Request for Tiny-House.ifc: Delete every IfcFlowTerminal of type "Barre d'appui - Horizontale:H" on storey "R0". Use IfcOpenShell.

First a look at what the model holds.

```python
import ifcopenshell
import ifcopenshell.util.element

model = ifcopenshell.open("Tiny-House.ifc")
print(model.schema)
storey = next(s for s in model.by_type("IfcBuildingStorey") if s.Name == "R0")
terminals = [e for e in ifcopenshell.util.element.get_decomposition(storey) if e.is_a("IfcFlowTerminal")]
seen = {}
for e in terminals:
    element_type = ifcopenshell.util.element.get_type(e)
    name = element_type.Name if element_type not in (None, e) else None
    seen[name] = seen.get(name, 0) + 1
for name, count in sorted(seen.items(), key=str):
    print(count, "x", name)
```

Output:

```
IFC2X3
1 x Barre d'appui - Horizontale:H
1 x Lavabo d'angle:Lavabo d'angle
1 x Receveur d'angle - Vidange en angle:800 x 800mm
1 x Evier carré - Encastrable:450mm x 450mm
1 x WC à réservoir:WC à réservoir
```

```python
import ifcopenshell
import ifcopenshell.api.root
import ifcopenshell.util.element

model = ifcopenshell.open("Tiny-House.ifc")

storey = next(s for s in model.by_type("IfcBuildingStorey") if s.Name == "R0")
terminals = [e for e in ifcopenshell.util.element.get_decomposition(storey) if e.is_a("IfcFlowTerminal")]
targets = [e for e in terminals if (t := ifcopenshell.util.element.get_type(e)) not in (None, e) and t.Name == "Barre d'appui - Horizontale:H"]

for e in targets:
    ifcopenshell.api.root.remove_product(model, product=e)
print(len(targets), "removed")

model.write("Tiny-House_rev.ifc")
```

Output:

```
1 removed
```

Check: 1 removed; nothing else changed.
